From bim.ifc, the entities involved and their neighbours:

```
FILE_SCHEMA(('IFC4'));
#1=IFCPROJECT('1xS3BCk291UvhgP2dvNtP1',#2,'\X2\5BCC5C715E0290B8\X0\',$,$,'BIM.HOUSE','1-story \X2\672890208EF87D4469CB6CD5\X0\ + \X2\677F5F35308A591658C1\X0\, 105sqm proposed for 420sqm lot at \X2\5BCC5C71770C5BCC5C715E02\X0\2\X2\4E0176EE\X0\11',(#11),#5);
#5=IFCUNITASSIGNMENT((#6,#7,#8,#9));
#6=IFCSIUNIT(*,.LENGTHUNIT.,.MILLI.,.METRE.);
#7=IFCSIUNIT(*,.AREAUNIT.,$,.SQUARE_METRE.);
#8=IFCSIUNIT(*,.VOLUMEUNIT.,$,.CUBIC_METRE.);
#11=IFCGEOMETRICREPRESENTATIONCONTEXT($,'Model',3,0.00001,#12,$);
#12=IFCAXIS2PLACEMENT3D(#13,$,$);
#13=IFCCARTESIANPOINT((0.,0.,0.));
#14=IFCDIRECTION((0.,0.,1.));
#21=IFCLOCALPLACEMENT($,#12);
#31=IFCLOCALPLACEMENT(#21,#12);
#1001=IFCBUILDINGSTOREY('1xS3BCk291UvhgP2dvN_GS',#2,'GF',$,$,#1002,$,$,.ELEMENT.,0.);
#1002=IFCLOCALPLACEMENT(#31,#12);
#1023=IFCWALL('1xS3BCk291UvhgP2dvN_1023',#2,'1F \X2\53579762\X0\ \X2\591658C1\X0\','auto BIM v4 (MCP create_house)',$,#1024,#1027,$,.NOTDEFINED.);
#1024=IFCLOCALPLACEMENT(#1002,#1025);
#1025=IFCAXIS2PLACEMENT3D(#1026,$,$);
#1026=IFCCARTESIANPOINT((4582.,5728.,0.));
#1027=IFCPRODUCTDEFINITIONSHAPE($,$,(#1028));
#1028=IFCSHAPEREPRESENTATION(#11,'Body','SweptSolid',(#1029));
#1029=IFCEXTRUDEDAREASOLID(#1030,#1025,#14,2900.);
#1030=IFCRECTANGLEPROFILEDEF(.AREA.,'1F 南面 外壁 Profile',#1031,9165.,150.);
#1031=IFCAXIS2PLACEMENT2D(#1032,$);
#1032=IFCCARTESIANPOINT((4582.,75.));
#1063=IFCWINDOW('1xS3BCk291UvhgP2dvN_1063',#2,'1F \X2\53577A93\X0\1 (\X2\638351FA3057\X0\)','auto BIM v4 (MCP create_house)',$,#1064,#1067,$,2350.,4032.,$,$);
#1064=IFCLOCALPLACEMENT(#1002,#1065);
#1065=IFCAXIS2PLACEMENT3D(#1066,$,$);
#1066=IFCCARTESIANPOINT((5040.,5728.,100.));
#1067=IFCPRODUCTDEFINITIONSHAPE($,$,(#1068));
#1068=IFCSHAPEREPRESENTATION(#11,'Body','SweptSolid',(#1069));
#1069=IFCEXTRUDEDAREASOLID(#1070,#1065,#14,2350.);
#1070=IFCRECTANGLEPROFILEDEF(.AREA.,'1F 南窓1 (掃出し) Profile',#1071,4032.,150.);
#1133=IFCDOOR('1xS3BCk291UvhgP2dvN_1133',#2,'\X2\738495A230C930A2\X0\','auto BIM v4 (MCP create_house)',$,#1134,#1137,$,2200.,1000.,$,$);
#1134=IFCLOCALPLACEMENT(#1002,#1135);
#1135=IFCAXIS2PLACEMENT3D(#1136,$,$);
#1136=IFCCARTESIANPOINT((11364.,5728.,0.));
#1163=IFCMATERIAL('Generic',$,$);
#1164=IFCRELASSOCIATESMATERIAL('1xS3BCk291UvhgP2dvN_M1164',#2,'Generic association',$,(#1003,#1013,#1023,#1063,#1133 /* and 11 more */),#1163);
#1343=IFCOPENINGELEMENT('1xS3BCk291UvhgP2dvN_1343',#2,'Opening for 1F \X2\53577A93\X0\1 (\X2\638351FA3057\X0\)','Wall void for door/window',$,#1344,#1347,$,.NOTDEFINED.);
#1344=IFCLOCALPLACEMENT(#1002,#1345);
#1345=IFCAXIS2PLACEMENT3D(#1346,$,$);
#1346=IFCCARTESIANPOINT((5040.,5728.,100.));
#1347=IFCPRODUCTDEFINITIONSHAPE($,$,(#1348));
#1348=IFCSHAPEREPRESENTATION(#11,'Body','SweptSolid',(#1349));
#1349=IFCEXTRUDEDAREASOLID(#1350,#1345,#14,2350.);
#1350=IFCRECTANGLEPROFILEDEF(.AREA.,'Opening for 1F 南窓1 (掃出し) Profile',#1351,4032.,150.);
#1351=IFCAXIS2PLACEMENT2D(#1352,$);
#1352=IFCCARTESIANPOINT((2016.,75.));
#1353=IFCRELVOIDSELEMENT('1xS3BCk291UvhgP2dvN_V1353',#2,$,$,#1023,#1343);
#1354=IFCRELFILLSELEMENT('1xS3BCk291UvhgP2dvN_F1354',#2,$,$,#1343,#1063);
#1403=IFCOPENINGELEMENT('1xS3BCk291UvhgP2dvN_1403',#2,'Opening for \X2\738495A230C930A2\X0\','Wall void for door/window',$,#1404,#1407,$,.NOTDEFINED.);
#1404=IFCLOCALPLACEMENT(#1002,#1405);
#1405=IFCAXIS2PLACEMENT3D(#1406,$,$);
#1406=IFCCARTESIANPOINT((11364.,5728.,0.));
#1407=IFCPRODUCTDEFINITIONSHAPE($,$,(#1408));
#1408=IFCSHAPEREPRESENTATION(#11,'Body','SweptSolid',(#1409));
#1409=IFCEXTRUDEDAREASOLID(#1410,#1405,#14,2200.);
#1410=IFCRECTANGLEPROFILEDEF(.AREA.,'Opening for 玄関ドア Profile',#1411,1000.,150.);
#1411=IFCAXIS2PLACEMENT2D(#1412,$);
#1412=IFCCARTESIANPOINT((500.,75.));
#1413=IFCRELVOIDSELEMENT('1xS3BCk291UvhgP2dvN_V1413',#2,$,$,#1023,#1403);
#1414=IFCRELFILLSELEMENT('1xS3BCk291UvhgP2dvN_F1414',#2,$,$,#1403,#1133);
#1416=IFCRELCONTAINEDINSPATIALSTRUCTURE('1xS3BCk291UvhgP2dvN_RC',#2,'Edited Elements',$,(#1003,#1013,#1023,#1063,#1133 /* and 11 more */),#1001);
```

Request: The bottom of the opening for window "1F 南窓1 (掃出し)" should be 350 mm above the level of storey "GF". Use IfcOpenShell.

```python
import numpy as np
import ifcopenshell
import ifcopenshell.api.geometry
import ifcopenshell.geom
import ifcopenshell.util.element
import ifcopenshell.util.placement
import ifcopenshell.util.shape
import ifcopenshell.util.unit

model = ifcopenshell.open("bim.ifc")
unit_scale = ifcopenshell.util.unit.calculate_unit_scale(model)

window = model.by_guid("1xS3BCk291UvhgP2dvN_1063")
opening = window.FillsVoids[0].RelatingOpeningElement
storey = ifcopenshell.util.element.get_container(window, ifc_class="IfcBuildingStorey")
level = ifcopenshell.util.placement.get_local_placement(storey.ObjectPlacement)[2, 3]

# The opening's origin need not be at the sill, so measure its lowest point.
shape = ifcopenshell.geom.create_shape(ifcopenshell.geom.settings(), opening)
bottom = ifcopenshell.util.shape.get_shape_bottom_elevation(shape, shape.geometry) / unit_scale
dz = level + 0.35 / unit_scale - bottom

shift = np.array([0.0, 0.0, dz])
# The window is not placed relative to its opening, so move both.
for product in (opening, window):
    matrix = ifcopenshell.util.placement.get_local_placement(product.ObjectPlacement)
    matrix[:3, 3] += shift
    ifcopenshell.api.geometry.edit_object_placement(model, product=product, matrix=matrix, is_si=False)

print(f"moved by {dz * unit_scale:+.3f} m")

model.write("bim_rev.ifc")
```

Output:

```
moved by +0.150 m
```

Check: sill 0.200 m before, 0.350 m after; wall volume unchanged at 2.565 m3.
